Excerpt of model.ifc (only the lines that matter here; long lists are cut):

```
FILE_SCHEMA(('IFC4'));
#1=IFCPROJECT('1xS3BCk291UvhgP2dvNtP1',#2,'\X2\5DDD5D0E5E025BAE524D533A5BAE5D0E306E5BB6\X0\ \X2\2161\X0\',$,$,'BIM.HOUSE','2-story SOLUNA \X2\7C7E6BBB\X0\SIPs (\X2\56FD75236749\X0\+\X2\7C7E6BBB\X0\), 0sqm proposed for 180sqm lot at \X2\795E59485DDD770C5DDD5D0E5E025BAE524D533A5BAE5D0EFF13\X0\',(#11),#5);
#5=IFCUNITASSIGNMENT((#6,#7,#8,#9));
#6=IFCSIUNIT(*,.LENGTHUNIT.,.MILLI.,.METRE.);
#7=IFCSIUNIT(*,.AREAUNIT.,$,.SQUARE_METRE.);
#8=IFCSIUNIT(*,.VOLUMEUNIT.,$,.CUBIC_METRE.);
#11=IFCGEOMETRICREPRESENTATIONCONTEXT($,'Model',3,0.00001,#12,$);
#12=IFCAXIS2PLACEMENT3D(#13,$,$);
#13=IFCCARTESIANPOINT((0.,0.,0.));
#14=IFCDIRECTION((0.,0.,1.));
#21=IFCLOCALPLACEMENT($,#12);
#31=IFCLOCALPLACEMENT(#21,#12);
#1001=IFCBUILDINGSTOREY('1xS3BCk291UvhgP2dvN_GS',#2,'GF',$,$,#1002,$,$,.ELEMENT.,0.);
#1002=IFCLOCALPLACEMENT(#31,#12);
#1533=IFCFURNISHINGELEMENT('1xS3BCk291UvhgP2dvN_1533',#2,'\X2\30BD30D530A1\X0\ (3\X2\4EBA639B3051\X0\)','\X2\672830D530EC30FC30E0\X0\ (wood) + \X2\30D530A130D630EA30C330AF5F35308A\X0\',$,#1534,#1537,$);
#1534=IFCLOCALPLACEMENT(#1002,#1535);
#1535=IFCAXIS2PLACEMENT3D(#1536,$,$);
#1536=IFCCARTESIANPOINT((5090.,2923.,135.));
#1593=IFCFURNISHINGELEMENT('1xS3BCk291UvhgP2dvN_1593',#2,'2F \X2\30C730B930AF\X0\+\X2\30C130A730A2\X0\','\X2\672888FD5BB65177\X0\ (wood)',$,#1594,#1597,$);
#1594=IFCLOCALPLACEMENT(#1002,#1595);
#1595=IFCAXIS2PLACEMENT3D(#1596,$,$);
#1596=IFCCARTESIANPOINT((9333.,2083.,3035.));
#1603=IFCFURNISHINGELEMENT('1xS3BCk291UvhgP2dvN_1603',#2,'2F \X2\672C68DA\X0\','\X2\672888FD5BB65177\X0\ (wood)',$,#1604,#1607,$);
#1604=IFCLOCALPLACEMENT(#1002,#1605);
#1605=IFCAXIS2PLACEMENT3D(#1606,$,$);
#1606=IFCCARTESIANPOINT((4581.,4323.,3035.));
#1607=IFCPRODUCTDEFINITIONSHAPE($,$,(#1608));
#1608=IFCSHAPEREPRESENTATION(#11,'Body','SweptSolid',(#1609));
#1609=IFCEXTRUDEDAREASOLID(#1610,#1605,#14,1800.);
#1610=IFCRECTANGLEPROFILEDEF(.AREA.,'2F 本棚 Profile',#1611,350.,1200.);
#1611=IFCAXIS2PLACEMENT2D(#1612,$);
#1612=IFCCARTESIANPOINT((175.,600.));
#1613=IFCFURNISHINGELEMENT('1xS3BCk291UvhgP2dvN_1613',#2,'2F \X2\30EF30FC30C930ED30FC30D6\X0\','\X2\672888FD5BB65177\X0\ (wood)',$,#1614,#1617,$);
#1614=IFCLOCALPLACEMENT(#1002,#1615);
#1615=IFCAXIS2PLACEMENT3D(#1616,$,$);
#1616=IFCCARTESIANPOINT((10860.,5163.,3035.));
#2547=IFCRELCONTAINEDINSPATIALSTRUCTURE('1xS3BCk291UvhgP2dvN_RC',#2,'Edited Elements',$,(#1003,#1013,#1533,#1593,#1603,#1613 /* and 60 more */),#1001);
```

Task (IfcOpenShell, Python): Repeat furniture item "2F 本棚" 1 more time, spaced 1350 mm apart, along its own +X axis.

```python
import ifcopenshell
import ifcopenshell.api.geometry
import ifcopenshell.api.root
import ifcopenshell.util.element
import ifcopenshell.util.placement

model = ifcopenshell.open("model.ifc")


def reuse_history(source, copy):
    """copy_class also copies each property set's owner history, people and application; keep the originals."""
    for rel in copy.IsDefinedBy:
        if rel.is_a("IfcRelDefinesByProperties") and (history := rel.RelatingPropertyDefinition.OwnerHistory):
            rel.RelatingPropertyDefinition.OwnerHistory = source.OwnerHistory
            ifcopenshell.util.element.remove_deep2(model, history)


source = model.by_guid("1xS3BCk291UvhgP2dvN_1603")
base = ifcopenshell.util.placement.get_local_placement(source.ObjectPlacement)
step = base[:3, 0] * 1350.0

for i in range(1, 2):
    copy = ifcopenshell.api.root.copy_class(model, product=source)
    copy.Representation = ifcopenshell.util.element.copy_deep(
        model, source.Representation, exclude=["IfcGeometricRepresentationContext", "IfcRepresentationMap"]
    )
    reuse_history(source, copy)
    matrix = base.copy()
    matrix[:3, 3] += i * step
    print("added at", matrix[:3, 3].round(3) + 0.0)
    ifcopenshell.api.geometry.edit_object_placement(model, product=copy, matrix=matrix, is_si=False)

model.write("model_updated.ifc")
```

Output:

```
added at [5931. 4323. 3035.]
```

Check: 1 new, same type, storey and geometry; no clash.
